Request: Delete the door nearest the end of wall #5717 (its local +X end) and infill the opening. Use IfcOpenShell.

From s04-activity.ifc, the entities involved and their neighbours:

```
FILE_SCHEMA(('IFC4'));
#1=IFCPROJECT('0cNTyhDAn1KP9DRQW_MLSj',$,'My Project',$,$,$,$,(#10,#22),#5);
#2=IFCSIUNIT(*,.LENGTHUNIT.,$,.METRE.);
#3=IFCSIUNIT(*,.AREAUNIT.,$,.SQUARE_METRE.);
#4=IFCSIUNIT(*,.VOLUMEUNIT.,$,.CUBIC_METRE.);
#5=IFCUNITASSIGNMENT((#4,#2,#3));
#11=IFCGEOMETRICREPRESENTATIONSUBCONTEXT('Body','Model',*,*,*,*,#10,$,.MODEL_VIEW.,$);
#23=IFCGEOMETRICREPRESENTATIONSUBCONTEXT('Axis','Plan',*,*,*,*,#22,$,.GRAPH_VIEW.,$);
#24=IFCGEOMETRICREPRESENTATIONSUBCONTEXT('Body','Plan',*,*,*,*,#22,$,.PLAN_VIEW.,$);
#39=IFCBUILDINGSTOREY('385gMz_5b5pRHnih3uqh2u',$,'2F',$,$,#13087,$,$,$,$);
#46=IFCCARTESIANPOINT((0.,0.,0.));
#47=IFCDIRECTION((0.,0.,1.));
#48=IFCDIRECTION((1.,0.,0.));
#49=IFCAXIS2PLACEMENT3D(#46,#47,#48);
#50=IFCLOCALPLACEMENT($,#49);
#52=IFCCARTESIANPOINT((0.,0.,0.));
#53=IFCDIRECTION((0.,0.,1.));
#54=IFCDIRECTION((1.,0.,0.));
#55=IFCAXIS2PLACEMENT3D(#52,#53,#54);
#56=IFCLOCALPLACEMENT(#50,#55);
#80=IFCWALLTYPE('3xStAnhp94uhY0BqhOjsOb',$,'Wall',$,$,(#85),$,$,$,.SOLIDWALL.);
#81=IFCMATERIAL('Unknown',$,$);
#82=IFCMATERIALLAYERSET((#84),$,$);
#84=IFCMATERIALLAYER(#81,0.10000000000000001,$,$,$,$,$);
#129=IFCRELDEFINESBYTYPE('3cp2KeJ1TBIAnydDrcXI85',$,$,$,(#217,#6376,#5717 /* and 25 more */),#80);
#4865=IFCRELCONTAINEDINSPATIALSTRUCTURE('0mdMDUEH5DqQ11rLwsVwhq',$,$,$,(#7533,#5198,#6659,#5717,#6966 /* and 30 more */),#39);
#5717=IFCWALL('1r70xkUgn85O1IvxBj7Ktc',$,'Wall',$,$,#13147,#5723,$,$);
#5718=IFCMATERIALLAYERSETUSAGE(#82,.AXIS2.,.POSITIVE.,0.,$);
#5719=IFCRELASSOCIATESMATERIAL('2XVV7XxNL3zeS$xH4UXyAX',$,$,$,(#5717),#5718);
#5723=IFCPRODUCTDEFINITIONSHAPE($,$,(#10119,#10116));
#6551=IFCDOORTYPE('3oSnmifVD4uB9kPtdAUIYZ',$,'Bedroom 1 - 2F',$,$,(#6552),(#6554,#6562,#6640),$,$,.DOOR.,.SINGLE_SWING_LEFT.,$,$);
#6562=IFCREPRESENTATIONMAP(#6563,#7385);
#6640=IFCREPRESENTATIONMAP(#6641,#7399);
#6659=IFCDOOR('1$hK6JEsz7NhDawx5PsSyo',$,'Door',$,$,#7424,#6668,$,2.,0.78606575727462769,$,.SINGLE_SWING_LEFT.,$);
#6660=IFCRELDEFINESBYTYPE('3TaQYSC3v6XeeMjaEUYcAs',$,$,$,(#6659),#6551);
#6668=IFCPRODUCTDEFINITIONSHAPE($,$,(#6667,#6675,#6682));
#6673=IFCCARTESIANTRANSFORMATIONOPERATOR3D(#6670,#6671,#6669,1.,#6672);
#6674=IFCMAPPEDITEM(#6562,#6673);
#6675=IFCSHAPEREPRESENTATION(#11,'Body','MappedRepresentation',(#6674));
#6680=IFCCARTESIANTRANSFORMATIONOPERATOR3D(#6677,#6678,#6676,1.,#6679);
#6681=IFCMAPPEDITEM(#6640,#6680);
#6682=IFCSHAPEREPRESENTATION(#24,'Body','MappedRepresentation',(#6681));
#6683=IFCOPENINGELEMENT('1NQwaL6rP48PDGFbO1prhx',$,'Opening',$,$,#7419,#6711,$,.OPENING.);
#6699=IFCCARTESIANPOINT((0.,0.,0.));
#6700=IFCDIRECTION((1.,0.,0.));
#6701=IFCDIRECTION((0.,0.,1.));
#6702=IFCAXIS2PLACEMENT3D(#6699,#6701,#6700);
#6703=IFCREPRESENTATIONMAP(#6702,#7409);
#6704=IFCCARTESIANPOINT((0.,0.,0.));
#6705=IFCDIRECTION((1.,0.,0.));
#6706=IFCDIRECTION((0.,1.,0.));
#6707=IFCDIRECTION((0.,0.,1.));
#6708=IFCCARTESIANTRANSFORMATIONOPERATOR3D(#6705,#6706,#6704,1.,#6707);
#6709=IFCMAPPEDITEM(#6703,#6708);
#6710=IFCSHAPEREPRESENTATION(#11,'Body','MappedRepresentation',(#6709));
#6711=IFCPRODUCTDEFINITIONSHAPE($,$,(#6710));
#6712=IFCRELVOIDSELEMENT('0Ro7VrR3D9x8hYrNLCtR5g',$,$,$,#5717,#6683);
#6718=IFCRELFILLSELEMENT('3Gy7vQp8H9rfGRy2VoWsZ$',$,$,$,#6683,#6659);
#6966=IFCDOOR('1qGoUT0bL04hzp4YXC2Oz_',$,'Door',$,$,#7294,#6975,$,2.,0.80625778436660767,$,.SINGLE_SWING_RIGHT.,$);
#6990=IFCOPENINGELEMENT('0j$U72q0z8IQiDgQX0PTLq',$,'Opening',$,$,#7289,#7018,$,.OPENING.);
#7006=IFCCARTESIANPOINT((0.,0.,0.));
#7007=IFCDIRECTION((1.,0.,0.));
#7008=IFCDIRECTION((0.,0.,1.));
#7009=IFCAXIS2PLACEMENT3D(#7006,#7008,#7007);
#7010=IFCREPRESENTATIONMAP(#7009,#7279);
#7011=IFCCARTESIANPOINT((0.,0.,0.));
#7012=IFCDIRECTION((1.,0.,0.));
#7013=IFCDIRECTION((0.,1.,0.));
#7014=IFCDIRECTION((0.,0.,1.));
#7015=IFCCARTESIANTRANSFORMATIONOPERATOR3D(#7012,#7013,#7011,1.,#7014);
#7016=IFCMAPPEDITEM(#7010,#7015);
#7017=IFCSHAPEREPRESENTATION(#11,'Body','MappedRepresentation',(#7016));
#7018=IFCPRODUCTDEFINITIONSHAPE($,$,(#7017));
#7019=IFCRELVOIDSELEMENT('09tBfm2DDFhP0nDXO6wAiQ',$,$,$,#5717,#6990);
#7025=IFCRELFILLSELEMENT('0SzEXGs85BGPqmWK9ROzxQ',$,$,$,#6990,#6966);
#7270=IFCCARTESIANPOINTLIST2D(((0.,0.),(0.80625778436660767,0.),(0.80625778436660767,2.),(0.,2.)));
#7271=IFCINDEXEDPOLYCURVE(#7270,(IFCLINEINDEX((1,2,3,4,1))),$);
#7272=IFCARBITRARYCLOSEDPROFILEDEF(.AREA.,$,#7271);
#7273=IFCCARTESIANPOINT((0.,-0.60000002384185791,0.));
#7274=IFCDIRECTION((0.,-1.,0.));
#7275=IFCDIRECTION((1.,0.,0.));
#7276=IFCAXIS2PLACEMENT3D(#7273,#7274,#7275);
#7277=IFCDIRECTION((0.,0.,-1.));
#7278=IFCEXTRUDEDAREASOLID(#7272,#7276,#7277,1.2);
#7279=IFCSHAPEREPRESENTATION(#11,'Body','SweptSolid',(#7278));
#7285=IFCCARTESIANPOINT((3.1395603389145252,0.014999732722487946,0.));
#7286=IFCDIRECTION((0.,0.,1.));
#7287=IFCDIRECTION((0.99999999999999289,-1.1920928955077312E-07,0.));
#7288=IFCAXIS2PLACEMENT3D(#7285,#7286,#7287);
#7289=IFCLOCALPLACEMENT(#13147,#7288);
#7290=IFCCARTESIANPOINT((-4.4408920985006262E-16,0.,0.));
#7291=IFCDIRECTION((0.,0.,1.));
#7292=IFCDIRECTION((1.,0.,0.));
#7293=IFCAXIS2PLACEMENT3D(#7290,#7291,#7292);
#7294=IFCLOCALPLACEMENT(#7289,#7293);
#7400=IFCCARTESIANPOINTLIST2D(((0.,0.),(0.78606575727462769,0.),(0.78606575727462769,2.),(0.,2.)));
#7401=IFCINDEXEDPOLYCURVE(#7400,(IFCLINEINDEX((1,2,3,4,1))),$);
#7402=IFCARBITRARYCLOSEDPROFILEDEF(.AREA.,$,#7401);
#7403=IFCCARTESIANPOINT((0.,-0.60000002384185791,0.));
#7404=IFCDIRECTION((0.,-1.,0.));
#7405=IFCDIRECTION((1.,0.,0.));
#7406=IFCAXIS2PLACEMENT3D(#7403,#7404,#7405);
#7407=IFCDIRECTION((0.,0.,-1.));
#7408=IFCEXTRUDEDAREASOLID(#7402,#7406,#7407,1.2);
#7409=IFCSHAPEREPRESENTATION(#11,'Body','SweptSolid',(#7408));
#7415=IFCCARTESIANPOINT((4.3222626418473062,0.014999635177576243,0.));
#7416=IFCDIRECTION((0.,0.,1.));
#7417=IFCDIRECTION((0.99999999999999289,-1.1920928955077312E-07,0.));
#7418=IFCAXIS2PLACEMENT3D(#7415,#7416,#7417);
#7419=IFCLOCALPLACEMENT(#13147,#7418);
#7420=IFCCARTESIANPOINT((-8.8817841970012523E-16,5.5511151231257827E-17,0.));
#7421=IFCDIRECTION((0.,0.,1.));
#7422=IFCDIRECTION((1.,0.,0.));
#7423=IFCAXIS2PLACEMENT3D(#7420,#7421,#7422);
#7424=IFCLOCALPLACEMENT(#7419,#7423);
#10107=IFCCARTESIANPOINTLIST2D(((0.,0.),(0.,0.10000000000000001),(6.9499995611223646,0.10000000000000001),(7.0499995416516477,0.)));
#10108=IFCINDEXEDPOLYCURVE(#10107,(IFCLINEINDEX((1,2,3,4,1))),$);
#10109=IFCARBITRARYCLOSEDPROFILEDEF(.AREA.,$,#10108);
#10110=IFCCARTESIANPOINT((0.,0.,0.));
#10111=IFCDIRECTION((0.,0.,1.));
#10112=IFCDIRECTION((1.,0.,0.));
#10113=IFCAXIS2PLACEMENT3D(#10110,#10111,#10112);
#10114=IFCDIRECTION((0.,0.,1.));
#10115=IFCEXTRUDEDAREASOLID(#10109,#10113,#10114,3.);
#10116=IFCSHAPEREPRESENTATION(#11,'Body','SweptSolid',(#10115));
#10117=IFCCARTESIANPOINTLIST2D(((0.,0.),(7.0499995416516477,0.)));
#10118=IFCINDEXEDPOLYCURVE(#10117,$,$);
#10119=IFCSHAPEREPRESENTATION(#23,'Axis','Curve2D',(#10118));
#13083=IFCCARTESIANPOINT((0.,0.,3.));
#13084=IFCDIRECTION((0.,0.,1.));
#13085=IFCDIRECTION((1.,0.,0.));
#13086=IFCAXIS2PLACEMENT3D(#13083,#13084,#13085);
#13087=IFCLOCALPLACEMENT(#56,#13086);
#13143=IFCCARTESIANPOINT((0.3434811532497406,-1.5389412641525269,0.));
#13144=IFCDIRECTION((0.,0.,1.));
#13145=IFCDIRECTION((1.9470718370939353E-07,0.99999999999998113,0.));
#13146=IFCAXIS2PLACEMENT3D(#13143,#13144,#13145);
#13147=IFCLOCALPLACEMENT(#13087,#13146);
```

```python
import ifcopenshell
import ifcopenshell.api.feature
import ifcopenshell.api.root
import ifcopenshell.geom
import ifcopenshell.util.shape

model = ifcopenshell.open("s04-activity.ifc")
settings = ifcopenshell.geom.settings()


def volume(element):
    """Net volume in cubic metres, openings subtracted."""
    shape = ifcopenshell.geom.create_shape(settings, element)
    return ifcopenshell.util.shape.get_volume(shape.geometry)


door = model.by_guid("1$hK6JEsz7NhDawx5PsSyo")
opening = door.FillsVoids[0].RelatingOpeningElement
wall = opening.VoidsElements[0].RelatingBuildingElement
before = volume(wall)

ifcopenshell.api.root.remove_product(model, product=door)
ifcopenshell.api.feature.remove_feature(model, feature=opening)

after = volume(wall)

print(f"wall volume {before:.3f} -> {after:.3f} m3")

model.write("s04-activity-out.ifc")
```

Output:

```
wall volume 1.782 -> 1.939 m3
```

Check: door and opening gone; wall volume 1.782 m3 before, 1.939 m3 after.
